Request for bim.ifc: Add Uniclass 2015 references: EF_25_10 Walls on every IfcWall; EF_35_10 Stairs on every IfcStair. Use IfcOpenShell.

First a look at what the model holds.

```python
import ifcopenshell

model = ifcopenshell.open("bim.ifc")
print(model.schema)
print("classifications:", [c.Name for c in model.by_type("IfcClassification")])
for ifc_class in ("IfcDoor", "IfcRoof", "IfcStair", "IfcWall", "IfcWindow"):
    print(ifc_class, len(model.by_type(ifc_class)))
```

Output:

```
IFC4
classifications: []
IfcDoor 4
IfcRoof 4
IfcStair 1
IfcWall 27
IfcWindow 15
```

```python
import ifcopenshell
import ifcopenshell.api.classification

model = ifcopenshell.open("bim.ifc")

system = ifcopenshell.api.classification.add_classification(model, classification="Uniclass 2015")

codes = {
    "IfcWall": ("EF_25_10", "Walls"),
    "IfcStair": ("EF_35_10", "Stairs"),
}
for ifc_class, (code, name) in codes.items():
    products = model.by_type(ifc_class)
    ifcopenshell.api.classification.add_reference(
        model, products=products, classification=system, identification=code, name=name
    )
    print(code, len(products))

model.write("bim-out.ifc")
```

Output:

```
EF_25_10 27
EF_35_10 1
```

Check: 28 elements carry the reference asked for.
